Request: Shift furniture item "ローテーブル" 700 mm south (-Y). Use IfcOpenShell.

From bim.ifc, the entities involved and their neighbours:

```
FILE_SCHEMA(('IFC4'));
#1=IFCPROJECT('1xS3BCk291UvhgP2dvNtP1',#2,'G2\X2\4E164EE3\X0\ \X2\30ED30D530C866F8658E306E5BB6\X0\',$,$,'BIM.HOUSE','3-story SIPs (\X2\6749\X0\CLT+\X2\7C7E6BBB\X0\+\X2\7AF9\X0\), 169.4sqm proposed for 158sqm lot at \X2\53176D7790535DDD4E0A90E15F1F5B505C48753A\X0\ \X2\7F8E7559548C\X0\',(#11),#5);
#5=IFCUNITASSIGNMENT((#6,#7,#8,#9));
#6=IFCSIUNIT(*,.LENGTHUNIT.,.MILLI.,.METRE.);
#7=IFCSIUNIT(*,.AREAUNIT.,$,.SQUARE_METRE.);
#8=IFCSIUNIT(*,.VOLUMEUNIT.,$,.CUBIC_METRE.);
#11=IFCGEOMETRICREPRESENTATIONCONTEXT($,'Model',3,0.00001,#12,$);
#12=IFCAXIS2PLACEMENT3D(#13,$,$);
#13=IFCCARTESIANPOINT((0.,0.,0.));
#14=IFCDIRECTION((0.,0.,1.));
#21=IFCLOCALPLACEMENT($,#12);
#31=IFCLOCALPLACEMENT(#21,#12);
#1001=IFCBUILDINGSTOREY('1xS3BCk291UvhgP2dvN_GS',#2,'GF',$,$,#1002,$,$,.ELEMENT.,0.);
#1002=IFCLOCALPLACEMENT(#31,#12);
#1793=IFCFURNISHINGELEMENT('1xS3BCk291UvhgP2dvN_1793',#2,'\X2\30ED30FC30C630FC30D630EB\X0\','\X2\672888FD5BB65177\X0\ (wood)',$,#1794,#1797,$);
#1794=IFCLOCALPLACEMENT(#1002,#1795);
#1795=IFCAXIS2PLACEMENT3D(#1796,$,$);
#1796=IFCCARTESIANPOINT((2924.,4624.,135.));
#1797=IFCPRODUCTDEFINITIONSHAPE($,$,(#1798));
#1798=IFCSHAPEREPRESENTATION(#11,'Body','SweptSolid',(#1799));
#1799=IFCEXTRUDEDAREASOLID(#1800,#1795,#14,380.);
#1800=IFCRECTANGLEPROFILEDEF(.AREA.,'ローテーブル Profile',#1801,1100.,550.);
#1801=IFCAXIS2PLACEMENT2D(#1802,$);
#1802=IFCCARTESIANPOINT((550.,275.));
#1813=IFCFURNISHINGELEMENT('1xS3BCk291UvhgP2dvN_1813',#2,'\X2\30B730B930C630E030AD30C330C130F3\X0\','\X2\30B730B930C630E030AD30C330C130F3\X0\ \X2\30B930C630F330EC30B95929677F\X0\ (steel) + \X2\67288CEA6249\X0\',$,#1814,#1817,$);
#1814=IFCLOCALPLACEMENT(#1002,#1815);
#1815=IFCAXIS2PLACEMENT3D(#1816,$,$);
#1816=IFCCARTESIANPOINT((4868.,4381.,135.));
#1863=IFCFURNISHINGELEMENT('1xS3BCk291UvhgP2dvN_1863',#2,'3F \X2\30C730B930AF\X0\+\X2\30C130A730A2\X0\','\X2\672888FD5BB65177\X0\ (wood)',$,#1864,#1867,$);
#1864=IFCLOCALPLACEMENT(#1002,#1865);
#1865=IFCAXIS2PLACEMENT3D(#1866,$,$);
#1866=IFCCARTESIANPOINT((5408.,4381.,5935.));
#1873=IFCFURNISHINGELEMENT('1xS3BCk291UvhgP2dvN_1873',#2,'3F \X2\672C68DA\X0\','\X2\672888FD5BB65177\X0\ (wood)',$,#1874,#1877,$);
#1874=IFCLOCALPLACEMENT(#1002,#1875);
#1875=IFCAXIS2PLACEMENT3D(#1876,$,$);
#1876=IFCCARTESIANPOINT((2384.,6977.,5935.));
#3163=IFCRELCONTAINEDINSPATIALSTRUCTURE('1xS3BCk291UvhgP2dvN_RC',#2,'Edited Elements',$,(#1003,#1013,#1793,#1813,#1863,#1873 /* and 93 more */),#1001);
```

```python
import ifcopenshell
import ifcopenshell.api.geometry
import ifcopenshell.util.placement
import ifcopenshell.util.unit

model = ifcopenshell.open("bim.ifc")
unit_scale = ifcopenshell.util.unit.calculate_unit_scale(model)

item = model.by_guid("1xS3BCk291UvhgP2dvN_1793")
matrix = ifcopenshell.util.placement.get_local_placement(item.ObjectPlacement)
matrix[1, 3] -= 0.7 / unit_scale
ifcopenshell.api.geometry.edit_object_placement(model, product=item, matrix=matrix, is_si=False)

print(ifcopenshell.util.placement.get_local_placement(item.ObjectPlacement).round(3) + 0.0)

model.write("bim_edited.ifc")
```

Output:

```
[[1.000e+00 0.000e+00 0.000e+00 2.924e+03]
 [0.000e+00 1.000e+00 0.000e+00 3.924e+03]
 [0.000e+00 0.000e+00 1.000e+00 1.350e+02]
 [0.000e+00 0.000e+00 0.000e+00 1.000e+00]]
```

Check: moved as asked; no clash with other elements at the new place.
